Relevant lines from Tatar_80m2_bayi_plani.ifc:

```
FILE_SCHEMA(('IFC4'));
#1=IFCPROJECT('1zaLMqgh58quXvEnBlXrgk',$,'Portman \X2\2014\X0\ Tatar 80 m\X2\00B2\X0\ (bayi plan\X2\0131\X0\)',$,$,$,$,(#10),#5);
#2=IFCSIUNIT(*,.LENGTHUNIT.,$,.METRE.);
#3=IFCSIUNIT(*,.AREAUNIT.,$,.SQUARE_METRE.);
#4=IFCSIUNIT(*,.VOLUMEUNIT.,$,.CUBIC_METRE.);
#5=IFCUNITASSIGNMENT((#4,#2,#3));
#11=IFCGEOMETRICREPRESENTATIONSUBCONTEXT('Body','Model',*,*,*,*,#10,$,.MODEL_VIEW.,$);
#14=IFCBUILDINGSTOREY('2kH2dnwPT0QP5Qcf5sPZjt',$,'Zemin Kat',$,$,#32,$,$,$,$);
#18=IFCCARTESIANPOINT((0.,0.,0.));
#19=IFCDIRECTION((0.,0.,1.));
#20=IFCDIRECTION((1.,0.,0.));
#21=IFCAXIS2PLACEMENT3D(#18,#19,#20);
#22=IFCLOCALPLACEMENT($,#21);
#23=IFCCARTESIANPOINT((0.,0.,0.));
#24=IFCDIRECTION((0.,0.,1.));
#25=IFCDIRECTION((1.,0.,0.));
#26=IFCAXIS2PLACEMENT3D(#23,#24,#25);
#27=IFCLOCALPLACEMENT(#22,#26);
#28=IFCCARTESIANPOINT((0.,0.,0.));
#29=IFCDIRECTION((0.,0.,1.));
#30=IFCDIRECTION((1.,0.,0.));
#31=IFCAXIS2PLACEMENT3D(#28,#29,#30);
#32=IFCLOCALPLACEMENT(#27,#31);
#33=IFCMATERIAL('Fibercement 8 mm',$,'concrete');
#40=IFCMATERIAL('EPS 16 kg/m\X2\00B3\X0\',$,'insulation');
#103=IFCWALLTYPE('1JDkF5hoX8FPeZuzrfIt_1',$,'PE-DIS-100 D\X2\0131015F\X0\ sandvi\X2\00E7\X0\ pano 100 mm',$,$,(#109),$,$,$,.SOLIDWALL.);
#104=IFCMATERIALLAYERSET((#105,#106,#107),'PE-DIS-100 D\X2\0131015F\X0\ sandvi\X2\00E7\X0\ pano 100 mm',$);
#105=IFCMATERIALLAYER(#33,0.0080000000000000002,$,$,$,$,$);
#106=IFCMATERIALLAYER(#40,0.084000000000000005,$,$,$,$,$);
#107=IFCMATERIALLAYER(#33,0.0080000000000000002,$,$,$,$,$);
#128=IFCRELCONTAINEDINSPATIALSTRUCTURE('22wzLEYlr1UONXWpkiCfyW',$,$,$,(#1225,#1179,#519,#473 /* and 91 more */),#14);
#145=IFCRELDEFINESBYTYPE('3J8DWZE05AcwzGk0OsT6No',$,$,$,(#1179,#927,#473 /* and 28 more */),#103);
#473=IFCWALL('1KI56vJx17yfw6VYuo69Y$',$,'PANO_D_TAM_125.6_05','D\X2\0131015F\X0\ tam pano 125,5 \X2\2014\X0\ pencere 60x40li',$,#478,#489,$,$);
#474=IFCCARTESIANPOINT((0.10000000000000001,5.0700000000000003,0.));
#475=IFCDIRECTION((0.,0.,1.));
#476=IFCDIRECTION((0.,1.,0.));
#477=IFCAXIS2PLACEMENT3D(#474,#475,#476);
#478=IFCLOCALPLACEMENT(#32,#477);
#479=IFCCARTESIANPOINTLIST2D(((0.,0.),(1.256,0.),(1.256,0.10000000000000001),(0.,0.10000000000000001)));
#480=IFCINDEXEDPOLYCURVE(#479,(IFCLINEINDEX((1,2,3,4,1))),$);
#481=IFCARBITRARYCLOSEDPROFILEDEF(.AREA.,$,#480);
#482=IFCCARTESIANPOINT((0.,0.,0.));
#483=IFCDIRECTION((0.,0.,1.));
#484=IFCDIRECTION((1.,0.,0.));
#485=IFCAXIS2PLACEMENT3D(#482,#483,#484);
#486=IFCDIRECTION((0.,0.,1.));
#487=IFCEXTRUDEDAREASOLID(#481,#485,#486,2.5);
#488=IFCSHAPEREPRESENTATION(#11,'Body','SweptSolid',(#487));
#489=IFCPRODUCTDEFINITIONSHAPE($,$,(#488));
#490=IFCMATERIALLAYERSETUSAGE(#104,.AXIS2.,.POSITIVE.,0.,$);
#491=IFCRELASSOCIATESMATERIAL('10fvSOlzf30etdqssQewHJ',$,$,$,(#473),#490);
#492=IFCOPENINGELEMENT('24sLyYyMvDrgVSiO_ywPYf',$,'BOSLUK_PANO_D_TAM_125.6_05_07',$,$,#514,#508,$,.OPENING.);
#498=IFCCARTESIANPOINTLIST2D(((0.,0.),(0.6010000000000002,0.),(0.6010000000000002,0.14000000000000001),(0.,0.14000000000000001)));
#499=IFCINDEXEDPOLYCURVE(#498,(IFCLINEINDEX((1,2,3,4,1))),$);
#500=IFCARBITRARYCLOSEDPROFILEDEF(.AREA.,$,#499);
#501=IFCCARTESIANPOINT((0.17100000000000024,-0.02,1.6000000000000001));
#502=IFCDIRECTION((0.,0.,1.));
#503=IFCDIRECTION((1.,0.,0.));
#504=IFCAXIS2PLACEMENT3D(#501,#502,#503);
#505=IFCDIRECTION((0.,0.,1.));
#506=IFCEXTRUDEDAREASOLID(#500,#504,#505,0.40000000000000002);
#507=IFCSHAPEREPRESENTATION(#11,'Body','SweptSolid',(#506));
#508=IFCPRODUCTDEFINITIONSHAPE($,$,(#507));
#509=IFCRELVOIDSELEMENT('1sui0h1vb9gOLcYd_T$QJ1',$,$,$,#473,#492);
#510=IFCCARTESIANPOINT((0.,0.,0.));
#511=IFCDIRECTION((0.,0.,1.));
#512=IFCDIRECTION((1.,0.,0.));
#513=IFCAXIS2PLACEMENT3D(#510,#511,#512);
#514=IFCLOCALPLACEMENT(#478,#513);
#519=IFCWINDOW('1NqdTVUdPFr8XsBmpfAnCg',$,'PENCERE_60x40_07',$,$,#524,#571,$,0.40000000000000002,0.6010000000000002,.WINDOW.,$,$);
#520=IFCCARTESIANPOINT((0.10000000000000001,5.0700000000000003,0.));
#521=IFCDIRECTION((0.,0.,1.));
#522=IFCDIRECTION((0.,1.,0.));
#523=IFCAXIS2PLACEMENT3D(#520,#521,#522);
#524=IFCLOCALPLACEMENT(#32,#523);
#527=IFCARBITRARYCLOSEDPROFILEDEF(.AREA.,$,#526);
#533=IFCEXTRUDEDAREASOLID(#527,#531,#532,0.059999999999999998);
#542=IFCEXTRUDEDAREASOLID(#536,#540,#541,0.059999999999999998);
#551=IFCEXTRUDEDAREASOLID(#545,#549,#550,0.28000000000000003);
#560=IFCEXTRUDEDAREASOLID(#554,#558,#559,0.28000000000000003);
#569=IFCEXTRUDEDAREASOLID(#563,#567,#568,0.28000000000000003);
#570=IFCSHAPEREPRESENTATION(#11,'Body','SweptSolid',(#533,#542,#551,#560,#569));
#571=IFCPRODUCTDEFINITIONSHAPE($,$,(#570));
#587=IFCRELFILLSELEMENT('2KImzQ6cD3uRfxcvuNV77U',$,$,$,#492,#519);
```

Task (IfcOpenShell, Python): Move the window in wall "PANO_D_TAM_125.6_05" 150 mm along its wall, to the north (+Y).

```python
import ifcopenshell
import ifcopenshell.api.geometry
import ifcopenshell.util.placement
import ifcopenshell.util.unit

model = ifcopenshell.open("Tatar_80m2_bayi_plani.ifc")
unit_scale = ifcopenshell.util.unit.calculate_unit_scale(model)

window = model.by_guid("1NqdTVUdPFr8XsBmpfAnCg")
opening = window.FillsVoids[0].RelatingOpeningElement
wall = opening.VoidsElements[0].RelatingBuildingElement

wall_matrix = ifcopenshell.util.placement.get_local_placement(wall.ObjectPlacement)
shift = wall_matrix[:3, 0] * 0.15 / unit_scale
before = ifcopenshell.util.placement.get_local_placement(window.ObjectPlacement)[:3, 3].copy()

# The window is not placed relative to its opening, so move both.
for product in (opening, window):
    matrix = ifcopenshell.util.placement.get_local_placement(product.ObjectPlacement)
    matrix[:3, 3] += shift
    ifcopenshell.api.geometry.edit_object_placement(model, product=product, matrix=matrix, is_si=False)

after = ifcopenshell.util.placement.get_local_placement(window.ObjectPlacement)[:3, 3]
print("window moved by", (after - before).round(3) + 0.0)

model.write("Tatar_80m2_bayi_plani_v2.ifc")
```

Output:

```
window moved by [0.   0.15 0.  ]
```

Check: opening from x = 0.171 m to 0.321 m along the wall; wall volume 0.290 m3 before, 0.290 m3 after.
